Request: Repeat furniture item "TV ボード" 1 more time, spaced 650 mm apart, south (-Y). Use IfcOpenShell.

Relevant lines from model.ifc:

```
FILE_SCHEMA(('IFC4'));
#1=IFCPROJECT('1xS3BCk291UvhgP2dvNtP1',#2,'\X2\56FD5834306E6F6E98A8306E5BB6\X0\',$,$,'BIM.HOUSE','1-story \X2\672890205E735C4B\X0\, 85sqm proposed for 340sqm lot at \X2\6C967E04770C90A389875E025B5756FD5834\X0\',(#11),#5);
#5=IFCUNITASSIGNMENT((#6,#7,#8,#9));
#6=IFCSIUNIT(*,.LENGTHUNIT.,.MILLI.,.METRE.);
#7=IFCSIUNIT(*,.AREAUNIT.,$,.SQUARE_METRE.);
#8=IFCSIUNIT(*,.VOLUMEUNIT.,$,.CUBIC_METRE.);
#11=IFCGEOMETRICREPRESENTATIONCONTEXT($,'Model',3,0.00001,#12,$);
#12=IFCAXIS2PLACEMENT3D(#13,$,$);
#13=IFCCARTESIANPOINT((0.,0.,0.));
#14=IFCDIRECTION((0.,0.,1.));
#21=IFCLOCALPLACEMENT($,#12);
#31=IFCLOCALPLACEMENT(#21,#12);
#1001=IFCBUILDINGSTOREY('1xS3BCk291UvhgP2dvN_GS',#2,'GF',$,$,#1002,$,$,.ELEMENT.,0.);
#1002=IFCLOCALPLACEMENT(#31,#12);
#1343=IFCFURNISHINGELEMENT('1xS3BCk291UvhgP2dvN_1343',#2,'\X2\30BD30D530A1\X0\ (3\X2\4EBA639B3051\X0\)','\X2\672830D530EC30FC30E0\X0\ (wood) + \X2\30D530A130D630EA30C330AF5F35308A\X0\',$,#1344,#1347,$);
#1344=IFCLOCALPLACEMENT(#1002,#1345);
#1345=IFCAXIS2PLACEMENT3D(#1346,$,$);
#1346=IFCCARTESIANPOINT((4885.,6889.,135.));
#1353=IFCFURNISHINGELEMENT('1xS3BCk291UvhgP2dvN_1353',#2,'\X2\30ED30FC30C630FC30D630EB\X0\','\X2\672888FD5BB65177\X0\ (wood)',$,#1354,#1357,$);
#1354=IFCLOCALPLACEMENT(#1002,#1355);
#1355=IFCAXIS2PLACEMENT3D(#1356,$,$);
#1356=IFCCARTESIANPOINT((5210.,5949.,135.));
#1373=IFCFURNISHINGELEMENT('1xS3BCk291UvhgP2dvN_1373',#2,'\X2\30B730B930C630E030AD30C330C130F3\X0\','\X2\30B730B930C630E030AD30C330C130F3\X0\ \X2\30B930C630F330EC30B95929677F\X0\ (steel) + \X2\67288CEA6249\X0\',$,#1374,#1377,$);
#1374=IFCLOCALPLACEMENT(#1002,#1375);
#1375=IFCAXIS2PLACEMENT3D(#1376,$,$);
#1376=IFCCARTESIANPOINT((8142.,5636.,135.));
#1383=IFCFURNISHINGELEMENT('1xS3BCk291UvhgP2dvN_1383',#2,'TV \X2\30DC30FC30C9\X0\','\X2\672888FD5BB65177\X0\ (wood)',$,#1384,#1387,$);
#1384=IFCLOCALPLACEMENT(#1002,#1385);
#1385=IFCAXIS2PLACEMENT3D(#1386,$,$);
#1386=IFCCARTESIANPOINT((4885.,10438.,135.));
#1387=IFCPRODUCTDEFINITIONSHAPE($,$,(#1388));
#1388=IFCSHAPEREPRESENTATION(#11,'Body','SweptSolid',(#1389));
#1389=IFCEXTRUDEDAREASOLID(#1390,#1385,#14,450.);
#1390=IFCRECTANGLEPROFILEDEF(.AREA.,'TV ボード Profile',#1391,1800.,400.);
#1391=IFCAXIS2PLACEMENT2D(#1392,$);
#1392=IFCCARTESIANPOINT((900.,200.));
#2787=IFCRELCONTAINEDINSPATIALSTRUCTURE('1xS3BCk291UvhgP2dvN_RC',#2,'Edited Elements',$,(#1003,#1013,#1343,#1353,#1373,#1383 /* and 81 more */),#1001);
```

```python
import numpy as np
import ifcopenshell
import ifcopenshell.api.geometry
import ifcopenshell.api.root
import ifcopenshell.util.element
import ifcopenshell.util.placement
import ifcopenshell.util.unit

model = ifcopenshell.open("model.ifc")
unit_scale = ifcopenshell.util.unit.calculate_unit_scale(model)


def reuse_history(source, copy):
    """copy_class also copies each property set's owner history, people and application; keep the originals."""
    for rel in copy.IsDefinedBy:
        if rel.is_a("IfcRelDefinesByProperties") and (history := rel.RelatingPropertyDefinition.OwnerHistory):
            rel.RelatingPropertyDefinition.OwnerHistory = source.OwnerHistory
            ifcopenshell.util.element.remove_deep2(model, history)


source = model.by_id(1383)
base = ifcopenshell.util.placement.get_local_placement(source.ObjectPlacement)
step = np.array([0.0, -1.0, 0.0]) * 0.65 / unit_scale

for i in range(1, 2):
    copy = ifcopenshell.api.root.copy_class(model, product=source)
    copy.Representation = ifcopenshell.util.element.copy_deep(
        model, source.Representation, exclude=["IfcGeometricRepresentationContext", "IfcRepresentationMap"]
    )
    reuse_history(source, copy)
    matrix = base.copy()
    matrix[:3, 3] += i * step
    print("added at", matrix[:3, 3].round(3) + 0.0)
    ifcopenshell.api.geometry.edit_object_placement(model, product=copy, matrix=matrix, is_si=False)

model.write("model_v2.ifc")
```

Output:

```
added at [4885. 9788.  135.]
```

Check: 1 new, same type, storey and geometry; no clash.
